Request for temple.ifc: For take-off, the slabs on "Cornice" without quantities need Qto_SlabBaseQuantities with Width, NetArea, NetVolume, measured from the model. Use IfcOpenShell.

First a look at what the model holds.

```python
import ifcopenshell
import ifcopenshell.util.element
import ifcopenshell.util.unit

model = ifcopenshell.open("temple.ifc")
print(model.schema)
for unit_type in ("LENGTHUNIT", "AREAUNIT", "VOLUMEUNIT"):
    print(unit_type, ifcopenshell.util.unit.calculate_unit_scale(model, unit_type))
storey = next(s for s in model.by_type("IfcBuildingStorey") if s.Name == "Cornice")
slabs = [e for e in ifcopenshell.util.element.get_decomposition(storey) if e.is_a("IfcSlab")]
for e in sorted(slabs, key=lambda e: e.id()):
    print(e.id(), e.is_a(), e.Name, list(ifcopenshell.util.element.get_psets(e, qtos_only=True)), sep=" | ")
```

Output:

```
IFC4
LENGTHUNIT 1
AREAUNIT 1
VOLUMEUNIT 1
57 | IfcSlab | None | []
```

```python
import ifcopenshell
import ifcopenshell.api.pset
import ifcopenshell.geom
import ifcopenshell.util.element
import ifcopenshell.util.shape
import ifcopenshell.util.unit

model = ifcopenshell.open("temple.ifc")
unit_scale = ifcopenshell.util.unit.calculate_unit_scale(model)
area_scale = ifcopenshell.util.unit.calculate_unit_scale(model, "AREAUNIT")
volume_scale = ifcopenshell.util.unit.calculate_unit_scale(model, "VOLUMEUNIT")
settings = ifcopenshell.geom.settings()

storey = next(s for s in model.by_type("IfcBuildingStorey") if s.Name == "Cornice")
slabs = [e for e in ifcopenshell.util.element.get_decomposition(storey) if e.is_a("IfcSlab")]

for e in sorted(slabs, key=lambda e: e.id()):
    if ifcopenshell.util.element.get_psets(e, qtos_only=True, should_inherit=False):
        continue
    # Geometry comes back in metres, in the element's own axes.
    shape = ifcopenshell.geom.create_shape(settings, e)
    values = {
        "Width": ifcopenshell.util.shape.get_z(shape.geometry) / unit_scale,
        "NetArea": ifcopenshell.util.shape.get_footprint_area(shape.geometry) / area_scale,
        "NetVolume": ifcopenshell.util.shape.get_volume(shape.geometry) / volume_scale,
    }
    qto = ifcopenshell.api.pset.add_qto(model, product=e, name="Qto_SlabBaseQuantities")
    ifcopenshell.api.pset.edit_qto(model, qto=qto, properties=values)
    print(e.id(), {k: round(v, 3) for k, v in values.items()})

model.write("temple_v2.ifc")
```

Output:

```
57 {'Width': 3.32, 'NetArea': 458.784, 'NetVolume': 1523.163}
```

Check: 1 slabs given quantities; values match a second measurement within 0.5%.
